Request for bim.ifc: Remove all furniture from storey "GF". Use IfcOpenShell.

First a look at what the model holds.

```python
import ifcopenshell
import ifcopenshell.util.element

model = ifcopenshell.open("bim.ifc")
print(model.schema)
storey = next(s for s in model.by_type("IfcBuildingStorey") if s.Name == "GF")
furniture = [e for e in ifcopenshell.util.element.get_decomposition(storey) if e.is_a("IfcFurnishingElement")]
seen = {}
for e in furniture:
    element_type = ifcopenshell.util.element.get_type(e)
    name = element_type.Name if element_type not in (None, e) else None
    seen[name] = seen.get(name, 0) + 1
for name, count in sorted(seen.items(), key=str):
    print(count, "x", name)
```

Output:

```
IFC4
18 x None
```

```python
import ifcopenshell
import ifcopenshell.api.root
import ifcopenshell.util.element

model = ifcopenshell.open("bim.ifc")

storey = next(s for s in model.by_type("IfcBuildingStorey") if s.Name == "GF")
furniture = [e for e in ifcopenshell.util.element.get_decomposition(storey) if e.is_a("IfcFurnishingElement")]

for e in furniture:
    ifcopenshell.api.root.remove_product(model, product=e)
print(len(furniture), "removed")

model.write("bim_edited.ifc")
```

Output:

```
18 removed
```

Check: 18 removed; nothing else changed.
